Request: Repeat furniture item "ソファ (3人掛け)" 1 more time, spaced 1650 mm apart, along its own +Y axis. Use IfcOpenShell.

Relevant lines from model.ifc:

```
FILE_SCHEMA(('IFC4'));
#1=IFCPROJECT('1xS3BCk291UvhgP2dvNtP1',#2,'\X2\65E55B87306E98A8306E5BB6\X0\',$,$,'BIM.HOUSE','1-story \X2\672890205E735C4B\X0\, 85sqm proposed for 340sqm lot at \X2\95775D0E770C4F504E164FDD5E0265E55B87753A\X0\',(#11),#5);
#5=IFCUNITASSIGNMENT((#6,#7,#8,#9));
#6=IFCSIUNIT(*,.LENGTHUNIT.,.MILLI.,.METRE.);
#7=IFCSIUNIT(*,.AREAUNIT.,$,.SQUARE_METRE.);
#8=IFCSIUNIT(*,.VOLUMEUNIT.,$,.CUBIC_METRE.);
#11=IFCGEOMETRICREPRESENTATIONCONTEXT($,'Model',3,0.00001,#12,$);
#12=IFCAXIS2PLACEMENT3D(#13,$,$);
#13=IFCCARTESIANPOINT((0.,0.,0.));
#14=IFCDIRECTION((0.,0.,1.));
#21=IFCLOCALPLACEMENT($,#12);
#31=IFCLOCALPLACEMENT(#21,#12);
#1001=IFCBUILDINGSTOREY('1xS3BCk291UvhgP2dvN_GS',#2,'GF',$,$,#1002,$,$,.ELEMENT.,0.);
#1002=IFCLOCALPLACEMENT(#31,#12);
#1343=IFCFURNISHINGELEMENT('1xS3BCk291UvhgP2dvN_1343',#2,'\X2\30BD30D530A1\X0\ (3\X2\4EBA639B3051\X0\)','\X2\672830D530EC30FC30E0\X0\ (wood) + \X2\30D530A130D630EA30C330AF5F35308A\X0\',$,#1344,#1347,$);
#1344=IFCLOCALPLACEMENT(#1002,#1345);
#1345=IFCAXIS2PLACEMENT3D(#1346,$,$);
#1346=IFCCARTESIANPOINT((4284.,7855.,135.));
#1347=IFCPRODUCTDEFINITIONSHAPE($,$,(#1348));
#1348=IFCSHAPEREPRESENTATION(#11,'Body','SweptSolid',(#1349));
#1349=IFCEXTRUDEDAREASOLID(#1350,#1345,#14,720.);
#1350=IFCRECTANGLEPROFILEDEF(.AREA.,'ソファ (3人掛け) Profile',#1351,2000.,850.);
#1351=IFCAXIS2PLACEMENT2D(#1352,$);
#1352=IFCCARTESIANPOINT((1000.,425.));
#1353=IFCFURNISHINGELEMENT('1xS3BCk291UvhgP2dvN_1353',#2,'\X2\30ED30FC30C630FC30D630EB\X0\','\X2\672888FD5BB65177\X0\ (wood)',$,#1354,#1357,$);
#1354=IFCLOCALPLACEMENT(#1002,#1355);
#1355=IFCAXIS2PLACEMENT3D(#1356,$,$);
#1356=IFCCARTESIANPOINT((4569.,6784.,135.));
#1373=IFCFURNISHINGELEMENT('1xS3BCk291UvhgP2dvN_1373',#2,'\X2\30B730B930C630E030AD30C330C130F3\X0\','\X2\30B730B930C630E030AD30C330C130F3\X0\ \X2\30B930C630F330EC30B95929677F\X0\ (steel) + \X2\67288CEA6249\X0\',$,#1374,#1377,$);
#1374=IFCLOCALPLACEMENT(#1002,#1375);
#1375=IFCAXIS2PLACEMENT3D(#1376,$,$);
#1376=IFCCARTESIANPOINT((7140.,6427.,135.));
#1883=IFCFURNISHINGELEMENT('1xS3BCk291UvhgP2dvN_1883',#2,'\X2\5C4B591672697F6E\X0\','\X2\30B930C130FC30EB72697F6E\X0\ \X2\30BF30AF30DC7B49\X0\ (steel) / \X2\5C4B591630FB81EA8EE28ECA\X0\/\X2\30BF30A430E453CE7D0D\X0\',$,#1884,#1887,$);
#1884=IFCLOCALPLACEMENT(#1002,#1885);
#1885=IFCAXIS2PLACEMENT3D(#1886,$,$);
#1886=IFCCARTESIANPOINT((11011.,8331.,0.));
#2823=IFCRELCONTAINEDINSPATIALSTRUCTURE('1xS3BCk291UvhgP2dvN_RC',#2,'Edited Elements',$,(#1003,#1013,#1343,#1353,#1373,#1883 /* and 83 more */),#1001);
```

```python
import ifcopenshell
import ifcopenshell.api.geometry
import ifcopenshell.api.root
import ifcopenshell.util.element
import ifcopenshell.util.placement
import ifcopenshell.util.unit

model = ifcopenshell.open("model.ifc")
unit_scale = ifcopenshell.util.unit.calculate_unit_scale(model)


def reuse_history(source, copy):
    """copy_class also copies each property set's owner history, people and application; keep the originals."""
    for rel in copy.IsDefinedBy:
        if rel.is_a("IfcRelDefinesByProperties") and (history := rel.RelatingPropertyDefinition.OwnerHistory):
            rel.RelatingPropertyDefinition.OwnerHistory = source.OwnerHistory
            ifcopenshell.util.element.remove_deep2(model, history)


source = model.by_guid("1xS3BCk291UvhgP2dvN_1343")
base = ifcopenshell.util.placement.get_local_placement(source.ObjectPlacement)
step = base[:3, 1] * 1.65 / unit_scale

for i in range(1, 2):
    copy = ifcopenshell.api.root.copy_class(model, product=source)
    copy.Representation = ifcopenshell.util.element.copy_deep(
        model, source.Representation, exclude=["IfcGeometricRepresentationContext", "IfcRepresentationMap"]
    )
    reuse_history(source, copy)
    matrix = base.copy()
    matrix[:3, 3] += i * step
    print("added at", matrix[:3, 3].round(3) + 0.0)
    ifcopenshell.api.geometry.edit_object_placement(model, product=copy, matrix=matrix, is_si=False)

model.write("model_rev.ifc")
```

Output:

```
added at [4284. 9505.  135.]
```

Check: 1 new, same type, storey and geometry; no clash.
